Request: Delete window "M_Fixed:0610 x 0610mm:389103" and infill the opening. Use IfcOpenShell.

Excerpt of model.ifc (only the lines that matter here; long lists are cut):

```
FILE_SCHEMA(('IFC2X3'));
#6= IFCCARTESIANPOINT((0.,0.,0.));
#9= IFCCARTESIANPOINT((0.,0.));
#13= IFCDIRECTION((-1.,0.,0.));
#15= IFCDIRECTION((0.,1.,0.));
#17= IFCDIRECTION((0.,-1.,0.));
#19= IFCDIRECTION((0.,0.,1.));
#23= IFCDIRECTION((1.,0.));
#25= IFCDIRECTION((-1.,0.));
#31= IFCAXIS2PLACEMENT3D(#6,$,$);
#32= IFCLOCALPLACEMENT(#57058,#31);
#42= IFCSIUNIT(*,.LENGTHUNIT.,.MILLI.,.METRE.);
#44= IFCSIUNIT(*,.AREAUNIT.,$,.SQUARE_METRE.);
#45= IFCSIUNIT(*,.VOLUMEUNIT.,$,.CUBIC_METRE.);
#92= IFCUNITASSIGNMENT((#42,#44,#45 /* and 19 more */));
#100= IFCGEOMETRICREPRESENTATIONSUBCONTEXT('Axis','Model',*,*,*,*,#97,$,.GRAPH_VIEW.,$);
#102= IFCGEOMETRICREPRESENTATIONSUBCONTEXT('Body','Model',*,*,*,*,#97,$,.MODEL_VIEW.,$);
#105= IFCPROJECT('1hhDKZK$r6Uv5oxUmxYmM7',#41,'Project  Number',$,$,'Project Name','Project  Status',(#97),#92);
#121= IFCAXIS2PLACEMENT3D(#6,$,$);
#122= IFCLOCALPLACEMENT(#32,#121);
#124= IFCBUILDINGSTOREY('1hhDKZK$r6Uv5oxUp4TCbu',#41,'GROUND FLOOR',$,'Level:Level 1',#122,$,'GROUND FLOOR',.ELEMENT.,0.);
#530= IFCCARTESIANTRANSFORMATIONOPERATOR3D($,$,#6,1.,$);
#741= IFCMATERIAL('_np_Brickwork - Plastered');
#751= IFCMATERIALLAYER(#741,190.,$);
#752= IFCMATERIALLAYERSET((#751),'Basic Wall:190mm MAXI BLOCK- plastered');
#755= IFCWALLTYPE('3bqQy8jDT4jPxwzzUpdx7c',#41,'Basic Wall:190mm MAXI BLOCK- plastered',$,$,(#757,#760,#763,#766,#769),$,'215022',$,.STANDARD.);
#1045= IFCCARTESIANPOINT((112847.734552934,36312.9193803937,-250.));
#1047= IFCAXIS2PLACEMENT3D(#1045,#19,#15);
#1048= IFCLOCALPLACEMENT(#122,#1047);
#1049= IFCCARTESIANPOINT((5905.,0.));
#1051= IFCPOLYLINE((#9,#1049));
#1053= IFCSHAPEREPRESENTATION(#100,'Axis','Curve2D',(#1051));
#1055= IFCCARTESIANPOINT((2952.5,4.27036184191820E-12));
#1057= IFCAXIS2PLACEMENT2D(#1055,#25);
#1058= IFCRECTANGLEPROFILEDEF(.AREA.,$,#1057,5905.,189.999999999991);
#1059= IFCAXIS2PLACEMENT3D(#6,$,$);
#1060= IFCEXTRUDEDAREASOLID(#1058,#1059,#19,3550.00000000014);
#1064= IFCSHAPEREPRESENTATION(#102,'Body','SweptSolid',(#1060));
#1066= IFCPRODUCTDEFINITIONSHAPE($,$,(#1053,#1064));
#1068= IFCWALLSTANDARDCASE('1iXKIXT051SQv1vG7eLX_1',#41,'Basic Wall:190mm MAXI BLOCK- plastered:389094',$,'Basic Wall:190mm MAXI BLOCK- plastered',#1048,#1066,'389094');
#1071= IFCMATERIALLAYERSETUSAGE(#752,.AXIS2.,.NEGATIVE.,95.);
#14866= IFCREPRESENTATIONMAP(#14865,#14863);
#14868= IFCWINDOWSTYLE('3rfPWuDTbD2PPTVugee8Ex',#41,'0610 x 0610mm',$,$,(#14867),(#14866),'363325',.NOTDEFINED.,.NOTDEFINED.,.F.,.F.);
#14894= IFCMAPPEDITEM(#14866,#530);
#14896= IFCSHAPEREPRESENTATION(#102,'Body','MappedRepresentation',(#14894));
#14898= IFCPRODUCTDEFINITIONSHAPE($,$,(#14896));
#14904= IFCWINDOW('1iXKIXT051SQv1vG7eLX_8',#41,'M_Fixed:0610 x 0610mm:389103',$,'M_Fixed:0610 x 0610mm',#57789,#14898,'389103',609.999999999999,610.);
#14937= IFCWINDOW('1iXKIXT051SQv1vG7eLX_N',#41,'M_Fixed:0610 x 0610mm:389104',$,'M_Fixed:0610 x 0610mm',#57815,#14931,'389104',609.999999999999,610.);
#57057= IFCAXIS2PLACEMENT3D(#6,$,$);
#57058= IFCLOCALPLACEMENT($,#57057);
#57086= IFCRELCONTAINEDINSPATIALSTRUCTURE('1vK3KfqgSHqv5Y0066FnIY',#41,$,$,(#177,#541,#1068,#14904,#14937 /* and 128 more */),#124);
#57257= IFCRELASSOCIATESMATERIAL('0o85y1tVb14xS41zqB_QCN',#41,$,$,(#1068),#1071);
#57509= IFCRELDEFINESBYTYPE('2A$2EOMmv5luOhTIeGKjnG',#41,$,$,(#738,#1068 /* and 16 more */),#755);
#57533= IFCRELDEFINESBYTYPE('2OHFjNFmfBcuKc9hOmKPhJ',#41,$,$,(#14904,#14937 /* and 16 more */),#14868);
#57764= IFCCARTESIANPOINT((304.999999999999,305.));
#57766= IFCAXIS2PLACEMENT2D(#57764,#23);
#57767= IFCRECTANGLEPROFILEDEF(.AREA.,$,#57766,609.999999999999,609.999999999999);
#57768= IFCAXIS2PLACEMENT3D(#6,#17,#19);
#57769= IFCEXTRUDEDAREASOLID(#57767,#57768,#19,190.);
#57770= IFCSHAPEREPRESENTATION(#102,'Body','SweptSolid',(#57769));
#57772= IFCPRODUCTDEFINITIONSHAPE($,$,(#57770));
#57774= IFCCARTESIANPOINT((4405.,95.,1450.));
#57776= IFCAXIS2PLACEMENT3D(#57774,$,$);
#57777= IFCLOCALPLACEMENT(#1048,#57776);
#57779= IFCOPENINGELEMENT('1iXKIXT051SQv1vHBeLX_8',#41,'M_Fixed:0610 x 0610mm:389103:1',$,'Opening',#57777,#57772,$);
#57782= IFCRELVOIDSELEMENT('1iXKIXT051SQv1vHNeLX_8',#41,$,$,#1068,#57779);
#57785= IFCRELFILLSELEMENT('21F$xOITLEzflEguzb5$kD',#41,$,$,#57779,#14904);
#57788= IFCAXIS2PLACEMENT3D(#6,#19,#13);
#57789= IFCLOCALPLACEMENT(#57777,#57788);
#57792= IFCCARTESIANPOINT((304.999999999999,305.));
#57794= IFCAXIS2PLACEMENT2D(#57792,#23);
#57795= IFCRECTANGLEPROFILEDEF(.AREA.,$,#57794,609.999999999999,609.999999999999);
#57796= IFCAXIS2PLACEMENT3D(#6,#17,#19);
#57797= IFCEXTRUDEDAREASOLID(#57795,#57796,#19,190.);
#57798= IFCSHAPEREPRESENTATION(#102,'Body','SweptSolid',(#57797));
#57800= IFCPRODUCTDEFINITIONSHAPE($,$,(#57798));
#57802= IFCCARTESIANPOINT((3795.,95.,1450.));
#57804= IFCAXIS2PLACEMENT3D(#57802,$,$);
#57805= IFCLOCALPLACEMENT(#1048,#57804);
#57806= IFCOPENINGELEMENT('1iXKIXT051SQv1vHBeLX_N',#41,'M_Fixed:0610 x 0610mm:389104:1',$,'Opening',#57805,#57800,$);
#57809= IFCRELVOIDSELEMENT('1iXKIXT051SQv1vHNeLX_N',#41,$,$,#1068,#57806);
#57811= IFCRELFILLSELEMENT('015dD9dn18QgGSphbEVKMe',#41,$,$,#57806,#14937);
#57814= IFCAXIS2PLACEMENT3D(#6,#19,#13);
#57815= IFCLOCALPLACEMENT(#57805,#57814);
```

```python
import ifcopenshell
import ifcopenshell.api.feature
import ifcopenshell.api.root
import ifcopenshell.geom
import ifcopenshell.util.shape

model = ifcopenshell.open("model.ifc")
settings = ifcopenshell.geom.settings()


def volume(element):
    """Net volume in cubic metres, openings subtracted."""
    shape = ifcopenshell.geom.create_shape(settings, element)
    return ifcopenshell.util.shape.get_volume(shape.geometry)


window = model.by_guid("1iXKIXT051SQv1vG7eLX_8")
opening = window.FillsVoids[0].RelatingOpeningElement
wall = opening.VoidsElements[0].RelatingBuildingElement
before = volume(wall)

ifcopenshell.api.root.remove_product(model, product=window)
ifcopenshell.api.feature.remove_feature(model, feature=opening)

after = volume(wall)

print(f"wall volume {before:.3f} -> {after:.3f} m3")

model.write("model-out.ifc")
```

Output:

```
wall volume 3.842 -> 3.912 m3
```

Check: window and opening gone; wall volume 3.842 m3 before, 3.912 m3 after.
